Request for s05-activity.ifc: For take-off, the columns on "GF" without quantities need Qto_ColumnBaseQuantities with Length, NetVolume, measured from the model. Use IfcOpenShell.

First a look at what the model holds.

```python
import ifcopenshell
import ifcopenshell.util.element
import ifcopenshell.util.unit

model = ifcopenshell.open("s05-activity.ifc")
print(model.schema)
for unit_type in ("LENGTHUNIT", "AREAUNIT", "VOLUMEUNIT"):
    print(unit_type, ifcopenshell.util.unit.calculate_unit_scale(model, unit_type))
storey = next(s for s in model.by_type("IfcBuildingStorey") if s.Name == "GF")
columns = [e for e in ifcopenshell.util.element.get_decomposition(storey) if e.is_a("IfcColumn")]
for e in sorted(columns, key=lambda e: e.id()):
    print(e.id(), e.is_a(), e.Name, list(ifcopenshell.util.element.get_psets(e, qtos_only=True)), sep=" | ")
```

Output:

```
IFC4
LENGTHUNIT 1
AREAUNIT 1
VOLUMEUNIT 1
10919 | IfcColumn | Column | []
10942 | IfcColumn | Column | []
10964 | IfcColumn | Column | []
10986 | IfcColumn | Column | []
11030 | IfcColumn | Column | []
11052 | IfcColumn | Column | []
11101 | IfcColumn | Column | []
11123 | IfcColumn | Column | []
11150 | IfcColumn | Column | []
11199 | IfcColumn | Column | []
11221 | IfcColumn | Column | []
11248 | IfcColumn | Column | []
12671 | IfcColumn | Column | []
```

```python
import ifcopenshell
import ifcopenshell.api.pset
import ifcopenshell.geom
import ifcopenshell.util.element
import ifcopenshell.util.shape
import ifcopenshell.util.unit

model = ifcopenshell.open("s05-activity.ifc")
unit_scale = ifcopenshell.util.unit.calculate_unit_scale(model)
volume_scale = ifcopenshell.util.unit.calculate_unit_scale(model, "VOLUMEUNIT")
settings = ifcopenshell.geom.settings()

storey = next(s for s in model.by_type("IfcBuildingStorey") if s.Name == "GF")
columns = [e for e in ifcopenshell.util.element.get_decomposition(storey) if e.is_a("IfcColumn")]

for e in sorted(columns, key=lambda e: e.id()):
    if ifcopenshell.util.element.get_psets(e, qtos_only=True, should_inherit=False):
        continue
    # Geometry comes back in metres, in the element's own axes.
    shape = ifcopenshell.geom.create_shape(settings, e)
    values = {
        "Length": ifcopenshell.util.shape.get_z(shape.geometry) / unit_scale,
        "NetVolume": ifcopenshell.util.shape.get_volume(shape.geometry) / volume_scale,
    }
    qto = ifcopenshell.api.pset.add_qto(model, product=e, name="Qto_ColumnBaseQuantities")
    ifcopenshell.api.pset.edit_qto(model, qto=qto, properties=values)
    print(e.id(), {k: round(v, 3) for k, v in values.items()})

model.write("s05-activity_v2.ifc")
```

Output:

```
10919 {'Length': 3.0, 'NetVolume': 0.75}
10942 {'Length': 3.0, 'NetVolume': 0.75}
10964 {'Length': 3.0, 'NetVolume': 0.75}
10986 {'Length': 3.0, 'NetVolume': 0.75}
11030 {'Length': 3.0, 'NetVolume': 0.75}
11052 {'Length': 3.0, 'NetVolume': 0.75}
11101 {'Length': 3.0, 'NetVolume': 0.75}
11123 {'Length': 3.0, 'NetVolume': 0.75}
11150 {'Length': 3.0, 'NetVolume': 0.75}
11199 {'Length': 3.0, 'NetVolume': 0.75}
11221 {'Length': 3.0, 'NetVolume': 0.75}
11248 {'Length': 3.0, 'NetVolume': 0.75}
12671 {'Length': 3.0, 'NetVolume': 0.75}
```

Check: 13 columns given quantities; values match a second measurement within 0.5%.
